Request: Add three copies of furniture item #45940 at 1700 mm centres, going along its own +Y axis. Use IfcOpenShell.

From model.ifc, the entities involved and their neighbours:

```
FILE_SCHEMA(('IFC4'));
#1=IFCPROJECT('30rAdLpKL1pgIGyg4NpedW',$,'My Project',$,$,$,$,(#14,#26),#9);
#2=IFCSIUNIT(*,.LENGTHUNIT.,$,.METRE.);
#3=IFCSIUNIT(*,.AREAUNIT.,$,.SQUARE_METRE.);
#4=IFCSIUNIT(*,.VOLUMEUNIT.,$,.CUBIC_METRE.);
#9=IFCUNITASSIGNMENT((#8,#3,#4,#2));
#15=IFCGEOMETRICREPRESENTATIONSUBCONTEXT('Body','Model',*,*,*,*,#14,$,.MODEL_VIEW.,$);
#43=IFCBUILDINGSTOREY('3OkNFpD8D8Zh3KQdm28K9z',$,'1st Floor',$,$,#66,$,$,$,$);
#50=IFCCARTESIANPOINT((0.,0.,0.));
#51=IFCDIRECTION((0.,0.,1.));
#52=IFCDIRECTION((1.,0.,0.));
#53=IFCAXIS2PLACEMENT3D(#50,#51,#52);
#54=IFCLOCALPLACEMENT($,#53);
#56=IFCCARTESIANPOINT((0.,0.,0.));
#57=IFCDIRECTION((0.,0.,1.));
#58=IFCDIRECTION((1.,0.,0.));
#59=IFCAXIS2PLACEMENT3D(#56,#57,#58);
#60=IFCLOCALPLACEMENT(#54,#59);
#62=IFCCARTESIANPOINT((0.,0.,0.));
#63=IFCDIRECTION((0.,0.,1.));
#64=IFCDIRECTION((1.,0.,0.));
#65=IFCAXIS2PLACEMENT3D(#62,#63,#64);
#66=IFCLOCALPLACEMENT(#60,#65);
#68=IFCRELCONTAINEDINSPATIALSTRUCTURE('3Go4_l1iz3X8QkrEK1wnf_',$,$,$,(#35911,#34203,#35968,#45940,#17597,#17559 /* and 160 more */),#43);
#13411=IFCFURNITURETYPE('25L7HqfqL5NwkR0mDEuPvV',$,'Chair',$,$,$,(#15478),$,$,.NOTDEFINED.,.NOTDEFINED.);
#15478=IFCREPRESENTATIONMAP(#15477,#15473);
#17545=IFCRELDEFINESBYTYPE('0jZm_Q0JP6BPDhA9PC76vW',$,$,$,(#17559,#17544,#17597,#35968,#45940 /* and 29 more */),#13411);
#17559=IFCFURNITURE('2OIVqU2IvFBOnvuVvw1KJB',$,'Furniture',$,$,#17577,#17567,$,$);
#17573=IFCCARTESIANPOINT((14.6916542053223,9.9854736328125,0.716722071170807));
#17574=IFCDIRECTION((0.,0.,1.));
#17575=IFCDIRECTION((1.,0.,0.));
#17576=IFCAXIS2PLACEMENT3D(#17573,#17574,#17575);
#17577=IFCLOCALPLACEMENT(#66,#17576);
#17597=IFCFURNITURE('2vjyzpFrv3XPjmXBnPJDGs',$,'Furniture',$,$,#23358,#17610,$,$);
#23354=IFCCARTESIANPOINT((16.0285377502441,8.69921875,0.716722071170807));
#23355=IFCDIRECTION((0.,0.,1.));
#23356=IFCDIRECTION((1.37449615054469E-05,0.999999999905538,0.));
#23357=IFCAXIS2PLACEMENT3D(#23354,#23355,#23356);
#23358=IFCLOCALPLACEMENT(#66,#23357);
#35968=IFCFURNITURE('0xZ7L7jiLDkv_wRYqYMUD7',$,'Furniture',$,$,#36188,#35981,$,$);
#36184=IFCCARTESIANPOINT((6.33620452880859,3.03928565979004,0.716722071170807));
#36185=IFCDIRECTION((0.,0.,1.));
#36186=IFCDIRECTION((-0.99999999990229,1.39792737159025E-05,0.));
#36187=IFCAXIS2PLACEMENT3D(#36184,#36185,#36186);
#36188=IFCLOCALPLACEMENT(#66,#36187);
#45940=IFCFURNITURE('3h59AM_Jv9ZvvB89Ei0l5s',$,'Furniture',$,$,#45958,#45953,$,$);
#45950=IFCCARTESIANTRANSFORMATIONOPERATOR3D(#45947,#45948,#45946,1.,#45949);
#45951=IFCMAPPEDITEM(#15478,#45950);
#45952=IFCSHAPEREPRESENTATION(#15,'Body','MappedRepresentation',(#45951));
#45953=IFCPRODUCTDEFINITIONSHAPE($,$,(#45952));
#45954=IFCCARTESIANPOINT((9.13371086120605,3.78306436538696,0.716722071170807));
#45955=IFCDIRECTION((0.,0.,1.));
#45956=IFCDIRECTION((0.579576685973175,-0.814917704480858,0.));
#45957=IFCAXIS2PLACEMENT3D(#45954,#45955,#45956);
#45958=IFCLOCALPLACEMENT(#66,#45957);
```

```python
import ifcopenshell
import ifcopenshell.api.geometry
import ifcopenshell.api.root
import ifcopenshell.util.element
import ifcopenshell.util.placement

model = ifcopenshell.open("model.ifc")

source = model.by_guid("3h59AM_Jv9ZvvB89Ei0l5s")
base = ifcopenshell.util.placement.get_local_placement(source.ObjectPlacement)
step = base[:3, 1] * 1.7

for i in range(1, 4):
    copy = ifcopenshell.api.root.copy_class(model, product=source)
    copy.Representation = ifcopenshell.util.element.copy_deep(
        model, source.Representation, exclude=["IfcGeometricRepresentationContext", "IfcRepresentationMap"]
    )
    matrix = base.copy()
    matrix[:3, 3] += i * step
    print("added at", matrix[:3, 3].round(3) + 0.0)
    ifcopenshell.api.geometry.edit_object_placement(model, product=copy, matrix=matrix, is_si=False)

model.write("model_v2.ifc")
```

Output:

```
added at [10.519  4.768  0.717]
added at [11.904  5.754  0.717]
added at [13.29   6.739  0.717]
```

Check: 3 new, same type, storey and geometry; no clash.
